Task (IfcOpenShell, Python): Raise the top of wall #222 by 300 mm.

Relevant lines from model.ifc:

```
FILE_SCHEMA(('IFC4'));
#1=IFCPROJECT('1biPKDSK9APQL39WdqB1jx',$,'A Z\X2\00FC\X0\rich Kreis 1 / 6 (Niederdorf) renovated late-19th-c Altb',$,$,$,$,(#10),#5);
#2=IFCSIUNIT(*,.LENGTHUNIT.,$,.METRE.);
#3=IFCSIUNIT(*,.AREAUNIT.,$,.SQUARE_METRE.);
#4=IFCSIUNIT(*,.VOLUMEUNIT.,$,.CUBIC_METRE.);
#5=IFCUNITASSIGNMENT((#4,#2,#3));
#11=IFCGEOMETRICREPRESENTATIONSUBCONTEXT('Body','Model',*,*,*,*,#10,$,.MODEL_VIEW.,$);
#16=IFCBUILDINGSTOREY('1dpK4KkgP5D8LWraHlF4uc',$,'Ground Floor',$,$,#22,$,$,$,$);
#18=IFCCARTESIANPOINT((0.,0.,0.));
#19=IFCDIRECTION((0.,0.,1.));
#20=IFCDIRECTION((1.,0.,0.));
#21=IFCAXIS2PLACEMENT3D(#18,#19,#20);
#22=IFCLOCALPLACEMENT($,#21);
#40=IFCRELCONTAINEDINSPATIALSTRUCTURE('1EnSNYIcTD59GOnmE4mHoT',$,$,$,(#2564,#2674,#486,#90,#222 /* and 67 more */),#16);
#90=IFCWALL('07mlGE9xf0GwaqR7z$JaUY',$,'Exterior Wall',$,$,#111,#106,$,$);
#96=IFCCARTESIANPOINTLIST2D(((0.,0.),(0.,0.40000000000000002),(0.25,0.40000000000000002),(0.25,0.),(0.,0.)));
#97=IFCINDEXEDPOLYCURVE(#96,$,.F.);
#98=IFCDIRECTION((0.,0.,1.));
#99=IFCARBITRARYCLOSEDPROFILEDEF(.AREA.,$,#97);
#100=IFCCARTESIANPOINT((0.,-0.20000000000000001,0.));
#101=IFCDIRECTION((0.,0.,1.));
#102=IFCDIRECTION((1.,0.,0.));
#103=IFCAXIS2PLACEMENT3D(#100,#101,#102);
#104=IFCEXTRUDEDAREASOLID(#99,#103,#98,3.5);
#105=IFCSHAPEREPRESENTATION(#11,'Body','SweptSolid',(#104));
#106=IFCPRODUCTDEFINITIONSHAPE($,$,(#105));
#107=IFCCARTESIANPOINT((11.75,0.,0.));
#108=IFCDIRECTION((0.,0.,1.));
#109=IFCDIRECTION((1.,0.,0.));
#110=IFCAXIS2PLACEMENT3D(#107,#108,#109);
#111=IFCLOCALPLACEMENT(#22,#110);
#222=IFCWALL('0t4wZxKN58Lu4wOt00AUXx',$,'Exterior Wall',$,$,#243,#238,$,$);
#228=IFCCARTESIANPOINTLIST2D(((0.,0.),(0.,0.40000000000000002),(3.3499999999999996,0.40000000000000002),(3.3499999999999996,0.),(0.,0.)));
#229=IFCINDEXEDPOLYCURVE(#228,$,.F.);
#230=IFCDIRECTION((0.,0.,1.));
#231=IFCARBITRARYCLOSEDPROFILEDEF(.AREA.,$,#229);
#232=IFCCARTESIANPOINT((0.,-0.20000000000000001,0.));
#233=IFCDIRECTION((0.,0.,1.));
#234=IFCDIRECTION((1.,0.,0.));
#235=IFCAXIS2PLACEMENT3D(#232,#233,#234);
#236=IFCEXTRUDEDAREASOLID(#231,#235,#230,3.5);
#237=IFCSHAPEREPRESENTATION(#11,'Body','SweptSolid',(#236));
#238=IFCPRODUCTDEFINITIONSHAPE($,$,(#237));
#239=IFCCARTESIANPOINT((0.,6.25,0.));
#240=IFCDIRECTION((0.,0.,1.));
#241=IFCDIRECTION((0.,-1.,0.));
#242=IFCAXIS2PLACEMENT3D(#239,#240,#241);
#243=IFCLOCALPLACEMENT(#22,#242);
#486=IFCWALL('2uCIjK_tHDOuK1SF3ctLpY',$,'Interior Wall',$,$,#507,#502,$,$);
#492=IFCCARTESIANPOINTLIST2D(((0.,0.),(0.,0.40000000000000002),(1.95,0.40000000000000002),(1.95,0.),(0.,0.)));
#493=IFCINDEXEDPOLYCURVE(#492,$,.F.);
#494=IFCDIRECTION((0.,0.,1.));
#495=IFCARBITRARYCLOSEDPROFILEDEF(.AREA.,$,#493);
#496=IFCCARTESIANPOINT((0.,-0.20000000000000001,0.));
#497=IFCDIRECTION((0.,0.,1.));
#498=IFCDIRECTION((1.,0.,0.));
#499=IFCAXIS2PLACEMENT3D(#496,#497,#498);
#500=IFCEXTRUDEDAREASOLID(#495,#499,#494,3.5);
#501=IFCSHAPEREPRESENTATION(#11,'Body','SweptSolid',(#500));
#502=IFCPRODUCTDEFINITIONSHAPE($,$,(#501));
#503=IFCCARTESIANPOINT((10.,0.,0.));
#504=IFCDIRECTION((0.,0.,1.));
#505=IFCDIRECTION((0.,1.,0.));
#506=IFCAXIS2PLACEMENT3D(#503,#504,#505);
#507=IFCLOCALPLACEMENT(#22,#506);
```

```python
import ifcopenshell
import ifcopenshell.geom
import ifcopenshell.util.representation
import ifcopenshell.util.shape
import ifcopenshell.util.unit

model = ifcopenshell.open("model.ifc")
unit_scale = ifcopenshell.util.unit.calculate_unit_scale(model)
settings = ifcopenshell.geom.settings()


def volume(element):
    """Net volume in cubic metres, openings subtracted."""
    shape = ifcopenshell.geom.create_shape(settings, element)
    return ifcopenshell.util.shape.get_volume(shape.geometry)


wall = model.by_guid("0t4wZxKN58Lu4wOt00AUXx")
before = volume(wall)

body = ifcopenshell.util.representation.get_representation(wall, "Model", "Body")
solid = body.Items[0]
old_height = solid.Depth
solid.Depth += 0.3 / unit_scale
after = volume(wall)

print(f"height {old_height:g} -> {solid.Depth:g}, volume {before:.3f} -> {after:.3f} m3")

model.write("model_edited.ifc")
```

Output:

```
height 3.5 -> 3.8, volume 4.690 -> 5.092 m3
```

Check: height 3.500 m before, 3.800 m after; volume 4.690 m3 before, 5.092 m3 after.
